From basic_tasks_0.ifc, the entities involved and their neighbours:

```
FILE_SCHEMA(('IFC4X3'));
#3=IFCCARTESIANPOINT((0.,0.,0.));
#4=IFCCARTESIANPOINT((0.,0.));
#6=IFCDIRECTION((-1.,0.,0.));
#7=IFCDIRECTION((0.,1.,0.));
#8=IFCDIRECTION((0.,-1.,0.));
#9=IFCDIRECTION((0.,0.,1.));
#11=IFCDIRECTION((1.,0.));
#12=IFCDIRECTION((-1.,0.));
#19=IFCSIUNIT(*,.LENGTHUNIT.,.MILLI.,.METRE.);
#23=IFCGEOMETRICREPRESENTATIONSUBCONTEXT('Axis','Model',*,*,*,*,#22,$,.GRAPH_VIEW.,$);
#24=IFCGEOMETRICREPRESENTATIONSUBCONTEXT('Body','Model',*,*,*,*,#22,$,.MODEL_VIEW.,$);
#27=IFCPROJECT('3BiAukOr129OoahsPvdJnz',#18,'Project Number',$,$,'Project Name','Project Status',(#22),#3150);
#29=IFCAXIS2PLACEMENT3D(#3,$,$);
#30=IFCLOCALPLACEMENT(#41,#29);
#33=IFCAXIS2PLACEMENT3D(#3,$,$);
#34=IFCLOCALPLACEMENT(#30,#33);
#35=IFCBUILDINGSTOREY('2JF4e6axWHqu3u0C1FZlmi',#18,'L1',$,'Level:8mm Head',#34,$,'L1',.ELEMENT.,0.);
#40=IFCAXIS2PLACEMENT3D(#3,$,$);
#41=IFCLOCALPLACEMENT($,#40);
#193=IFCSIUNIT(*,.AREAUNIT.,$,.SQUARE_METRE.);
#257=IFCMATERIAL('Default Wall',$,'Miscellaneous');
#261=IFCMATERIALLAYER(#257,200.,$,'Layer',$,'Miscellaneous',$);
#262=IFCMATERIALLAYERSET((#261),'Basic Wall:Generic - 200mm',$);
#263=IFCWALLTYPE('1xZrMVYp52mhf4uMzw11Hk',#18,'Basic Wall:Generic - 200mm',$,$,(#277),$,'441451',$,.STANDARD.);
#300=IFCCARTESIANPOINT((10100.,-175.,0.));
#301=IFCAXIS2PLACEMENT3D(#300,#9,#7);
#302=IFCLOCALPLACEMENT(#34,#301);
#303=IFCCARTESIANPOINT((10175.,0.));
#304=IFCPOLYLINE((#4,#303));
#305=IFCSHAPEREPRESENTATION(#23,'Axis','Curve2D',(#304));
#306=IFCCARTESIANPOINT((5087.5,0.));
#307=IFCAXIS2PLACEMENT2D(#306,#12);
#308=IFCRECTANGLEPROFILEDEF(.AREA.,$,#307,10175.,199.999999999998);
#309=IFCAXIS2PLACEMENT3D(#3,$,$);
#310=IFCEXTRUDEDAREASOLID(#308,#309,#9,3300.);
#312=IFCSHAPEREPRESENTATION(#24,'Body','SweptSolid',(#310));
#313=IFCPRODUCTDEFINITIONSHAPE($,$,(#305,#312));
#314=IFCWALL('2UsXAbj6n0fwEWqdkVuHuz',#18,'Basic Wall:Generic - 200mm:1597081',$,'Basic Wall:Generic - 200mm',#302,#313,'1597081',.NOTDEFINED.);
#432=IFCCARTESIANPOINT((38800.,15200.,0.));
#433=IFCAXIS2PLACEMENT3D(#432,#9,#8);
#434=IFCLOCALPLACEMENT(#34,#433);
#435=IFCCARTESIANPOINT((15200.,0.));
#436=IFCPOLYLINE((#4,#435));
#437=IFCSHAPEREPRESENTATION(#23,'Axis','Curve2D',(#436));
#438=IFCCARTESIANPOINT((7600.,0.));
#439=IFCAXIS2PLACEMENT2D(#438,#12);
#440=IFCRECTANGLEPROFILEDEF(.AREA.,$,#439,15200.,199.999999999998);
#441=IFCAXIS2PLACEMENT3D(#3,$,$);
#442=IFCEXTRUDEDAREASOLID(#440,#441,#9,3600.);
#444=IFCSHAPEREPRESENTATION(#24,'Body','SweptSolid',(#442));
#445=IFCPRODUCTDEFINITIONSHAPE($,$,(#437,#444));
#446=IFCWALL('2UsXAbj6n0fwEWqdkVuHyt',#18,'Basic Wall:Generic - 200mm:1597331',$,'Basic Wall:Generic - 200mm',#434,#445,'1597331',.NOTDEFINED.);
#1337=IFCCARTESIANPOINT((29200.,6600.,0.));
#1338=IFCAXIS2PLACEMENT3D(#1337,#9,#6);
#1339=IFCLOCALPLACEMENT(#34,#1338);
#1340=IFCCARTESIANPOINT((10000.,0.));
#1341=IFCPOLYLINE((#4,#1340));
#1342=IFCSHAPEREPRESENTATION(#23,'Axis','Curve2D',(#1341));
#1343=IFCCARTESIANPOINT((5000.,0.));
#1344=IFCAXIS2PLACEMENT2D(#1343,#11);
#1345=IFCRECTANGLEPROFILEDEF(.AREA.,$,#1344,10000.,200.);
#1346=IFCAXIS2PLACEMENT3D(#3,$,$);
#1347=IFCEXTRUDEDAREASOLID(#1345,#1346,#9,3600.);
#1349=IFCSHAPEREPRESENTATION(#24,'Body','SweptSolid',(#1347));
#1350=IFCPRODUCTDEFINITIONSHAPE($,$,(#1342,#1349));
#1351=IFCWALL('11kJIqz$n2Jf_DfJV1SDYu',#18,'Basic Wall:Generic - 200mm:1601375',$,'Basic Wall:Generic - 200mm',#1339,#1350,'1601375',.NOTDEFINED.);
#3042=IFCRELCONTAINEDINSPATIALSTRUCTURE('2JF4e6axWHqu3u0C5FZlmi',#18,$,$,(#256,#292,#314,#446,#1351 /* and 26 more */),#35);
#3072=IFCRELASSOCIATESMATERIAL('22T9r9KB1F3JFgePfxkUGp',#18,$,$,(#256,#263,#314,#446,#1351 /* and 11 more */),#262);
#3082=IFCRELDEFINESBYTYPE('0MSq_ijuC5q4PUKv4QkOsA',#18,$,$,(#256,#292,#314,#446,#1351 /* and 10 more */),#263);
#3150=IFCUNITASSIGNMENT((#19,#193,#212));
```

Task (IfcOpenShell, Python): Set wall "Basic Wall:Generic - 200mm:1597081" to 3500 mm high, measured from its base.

```python
import ifcopenshell
import ifcopenshell.geom
import ifcopenshell.util.representation
import ifcopenshell.util.shape

model = ifcopenshell.open("basic_tasks_0.ifc")
settings = ifcopenshell.geom.settings()


def volume(element):
    """Net volume in cubic metres, openings subtracted."""
    shape = ifcopenshell.geom.create_shape(settings, element)
    return ifcopenshell.util.shape.get_volume(shape.geometry)


wall = model.by_id(314)
before = volume(wall)

body = ifcopenshell.util.representation.get_representation(wall, "Model", "Body")
solid = body.Items[0]
old_height = solid.Depth
solid.Depth = 3500.0
after = volume(wall)

print(f"height {old_height:g} -> {solid.Depth:g}, volume {before:.3f} -> {after:.3f} m3")

model.write("basic_tasks_0_updated.ifc")
```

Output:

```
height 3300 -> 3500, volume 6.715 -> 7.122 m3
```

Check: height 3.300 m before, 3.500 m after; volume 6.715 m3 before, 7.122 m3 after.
